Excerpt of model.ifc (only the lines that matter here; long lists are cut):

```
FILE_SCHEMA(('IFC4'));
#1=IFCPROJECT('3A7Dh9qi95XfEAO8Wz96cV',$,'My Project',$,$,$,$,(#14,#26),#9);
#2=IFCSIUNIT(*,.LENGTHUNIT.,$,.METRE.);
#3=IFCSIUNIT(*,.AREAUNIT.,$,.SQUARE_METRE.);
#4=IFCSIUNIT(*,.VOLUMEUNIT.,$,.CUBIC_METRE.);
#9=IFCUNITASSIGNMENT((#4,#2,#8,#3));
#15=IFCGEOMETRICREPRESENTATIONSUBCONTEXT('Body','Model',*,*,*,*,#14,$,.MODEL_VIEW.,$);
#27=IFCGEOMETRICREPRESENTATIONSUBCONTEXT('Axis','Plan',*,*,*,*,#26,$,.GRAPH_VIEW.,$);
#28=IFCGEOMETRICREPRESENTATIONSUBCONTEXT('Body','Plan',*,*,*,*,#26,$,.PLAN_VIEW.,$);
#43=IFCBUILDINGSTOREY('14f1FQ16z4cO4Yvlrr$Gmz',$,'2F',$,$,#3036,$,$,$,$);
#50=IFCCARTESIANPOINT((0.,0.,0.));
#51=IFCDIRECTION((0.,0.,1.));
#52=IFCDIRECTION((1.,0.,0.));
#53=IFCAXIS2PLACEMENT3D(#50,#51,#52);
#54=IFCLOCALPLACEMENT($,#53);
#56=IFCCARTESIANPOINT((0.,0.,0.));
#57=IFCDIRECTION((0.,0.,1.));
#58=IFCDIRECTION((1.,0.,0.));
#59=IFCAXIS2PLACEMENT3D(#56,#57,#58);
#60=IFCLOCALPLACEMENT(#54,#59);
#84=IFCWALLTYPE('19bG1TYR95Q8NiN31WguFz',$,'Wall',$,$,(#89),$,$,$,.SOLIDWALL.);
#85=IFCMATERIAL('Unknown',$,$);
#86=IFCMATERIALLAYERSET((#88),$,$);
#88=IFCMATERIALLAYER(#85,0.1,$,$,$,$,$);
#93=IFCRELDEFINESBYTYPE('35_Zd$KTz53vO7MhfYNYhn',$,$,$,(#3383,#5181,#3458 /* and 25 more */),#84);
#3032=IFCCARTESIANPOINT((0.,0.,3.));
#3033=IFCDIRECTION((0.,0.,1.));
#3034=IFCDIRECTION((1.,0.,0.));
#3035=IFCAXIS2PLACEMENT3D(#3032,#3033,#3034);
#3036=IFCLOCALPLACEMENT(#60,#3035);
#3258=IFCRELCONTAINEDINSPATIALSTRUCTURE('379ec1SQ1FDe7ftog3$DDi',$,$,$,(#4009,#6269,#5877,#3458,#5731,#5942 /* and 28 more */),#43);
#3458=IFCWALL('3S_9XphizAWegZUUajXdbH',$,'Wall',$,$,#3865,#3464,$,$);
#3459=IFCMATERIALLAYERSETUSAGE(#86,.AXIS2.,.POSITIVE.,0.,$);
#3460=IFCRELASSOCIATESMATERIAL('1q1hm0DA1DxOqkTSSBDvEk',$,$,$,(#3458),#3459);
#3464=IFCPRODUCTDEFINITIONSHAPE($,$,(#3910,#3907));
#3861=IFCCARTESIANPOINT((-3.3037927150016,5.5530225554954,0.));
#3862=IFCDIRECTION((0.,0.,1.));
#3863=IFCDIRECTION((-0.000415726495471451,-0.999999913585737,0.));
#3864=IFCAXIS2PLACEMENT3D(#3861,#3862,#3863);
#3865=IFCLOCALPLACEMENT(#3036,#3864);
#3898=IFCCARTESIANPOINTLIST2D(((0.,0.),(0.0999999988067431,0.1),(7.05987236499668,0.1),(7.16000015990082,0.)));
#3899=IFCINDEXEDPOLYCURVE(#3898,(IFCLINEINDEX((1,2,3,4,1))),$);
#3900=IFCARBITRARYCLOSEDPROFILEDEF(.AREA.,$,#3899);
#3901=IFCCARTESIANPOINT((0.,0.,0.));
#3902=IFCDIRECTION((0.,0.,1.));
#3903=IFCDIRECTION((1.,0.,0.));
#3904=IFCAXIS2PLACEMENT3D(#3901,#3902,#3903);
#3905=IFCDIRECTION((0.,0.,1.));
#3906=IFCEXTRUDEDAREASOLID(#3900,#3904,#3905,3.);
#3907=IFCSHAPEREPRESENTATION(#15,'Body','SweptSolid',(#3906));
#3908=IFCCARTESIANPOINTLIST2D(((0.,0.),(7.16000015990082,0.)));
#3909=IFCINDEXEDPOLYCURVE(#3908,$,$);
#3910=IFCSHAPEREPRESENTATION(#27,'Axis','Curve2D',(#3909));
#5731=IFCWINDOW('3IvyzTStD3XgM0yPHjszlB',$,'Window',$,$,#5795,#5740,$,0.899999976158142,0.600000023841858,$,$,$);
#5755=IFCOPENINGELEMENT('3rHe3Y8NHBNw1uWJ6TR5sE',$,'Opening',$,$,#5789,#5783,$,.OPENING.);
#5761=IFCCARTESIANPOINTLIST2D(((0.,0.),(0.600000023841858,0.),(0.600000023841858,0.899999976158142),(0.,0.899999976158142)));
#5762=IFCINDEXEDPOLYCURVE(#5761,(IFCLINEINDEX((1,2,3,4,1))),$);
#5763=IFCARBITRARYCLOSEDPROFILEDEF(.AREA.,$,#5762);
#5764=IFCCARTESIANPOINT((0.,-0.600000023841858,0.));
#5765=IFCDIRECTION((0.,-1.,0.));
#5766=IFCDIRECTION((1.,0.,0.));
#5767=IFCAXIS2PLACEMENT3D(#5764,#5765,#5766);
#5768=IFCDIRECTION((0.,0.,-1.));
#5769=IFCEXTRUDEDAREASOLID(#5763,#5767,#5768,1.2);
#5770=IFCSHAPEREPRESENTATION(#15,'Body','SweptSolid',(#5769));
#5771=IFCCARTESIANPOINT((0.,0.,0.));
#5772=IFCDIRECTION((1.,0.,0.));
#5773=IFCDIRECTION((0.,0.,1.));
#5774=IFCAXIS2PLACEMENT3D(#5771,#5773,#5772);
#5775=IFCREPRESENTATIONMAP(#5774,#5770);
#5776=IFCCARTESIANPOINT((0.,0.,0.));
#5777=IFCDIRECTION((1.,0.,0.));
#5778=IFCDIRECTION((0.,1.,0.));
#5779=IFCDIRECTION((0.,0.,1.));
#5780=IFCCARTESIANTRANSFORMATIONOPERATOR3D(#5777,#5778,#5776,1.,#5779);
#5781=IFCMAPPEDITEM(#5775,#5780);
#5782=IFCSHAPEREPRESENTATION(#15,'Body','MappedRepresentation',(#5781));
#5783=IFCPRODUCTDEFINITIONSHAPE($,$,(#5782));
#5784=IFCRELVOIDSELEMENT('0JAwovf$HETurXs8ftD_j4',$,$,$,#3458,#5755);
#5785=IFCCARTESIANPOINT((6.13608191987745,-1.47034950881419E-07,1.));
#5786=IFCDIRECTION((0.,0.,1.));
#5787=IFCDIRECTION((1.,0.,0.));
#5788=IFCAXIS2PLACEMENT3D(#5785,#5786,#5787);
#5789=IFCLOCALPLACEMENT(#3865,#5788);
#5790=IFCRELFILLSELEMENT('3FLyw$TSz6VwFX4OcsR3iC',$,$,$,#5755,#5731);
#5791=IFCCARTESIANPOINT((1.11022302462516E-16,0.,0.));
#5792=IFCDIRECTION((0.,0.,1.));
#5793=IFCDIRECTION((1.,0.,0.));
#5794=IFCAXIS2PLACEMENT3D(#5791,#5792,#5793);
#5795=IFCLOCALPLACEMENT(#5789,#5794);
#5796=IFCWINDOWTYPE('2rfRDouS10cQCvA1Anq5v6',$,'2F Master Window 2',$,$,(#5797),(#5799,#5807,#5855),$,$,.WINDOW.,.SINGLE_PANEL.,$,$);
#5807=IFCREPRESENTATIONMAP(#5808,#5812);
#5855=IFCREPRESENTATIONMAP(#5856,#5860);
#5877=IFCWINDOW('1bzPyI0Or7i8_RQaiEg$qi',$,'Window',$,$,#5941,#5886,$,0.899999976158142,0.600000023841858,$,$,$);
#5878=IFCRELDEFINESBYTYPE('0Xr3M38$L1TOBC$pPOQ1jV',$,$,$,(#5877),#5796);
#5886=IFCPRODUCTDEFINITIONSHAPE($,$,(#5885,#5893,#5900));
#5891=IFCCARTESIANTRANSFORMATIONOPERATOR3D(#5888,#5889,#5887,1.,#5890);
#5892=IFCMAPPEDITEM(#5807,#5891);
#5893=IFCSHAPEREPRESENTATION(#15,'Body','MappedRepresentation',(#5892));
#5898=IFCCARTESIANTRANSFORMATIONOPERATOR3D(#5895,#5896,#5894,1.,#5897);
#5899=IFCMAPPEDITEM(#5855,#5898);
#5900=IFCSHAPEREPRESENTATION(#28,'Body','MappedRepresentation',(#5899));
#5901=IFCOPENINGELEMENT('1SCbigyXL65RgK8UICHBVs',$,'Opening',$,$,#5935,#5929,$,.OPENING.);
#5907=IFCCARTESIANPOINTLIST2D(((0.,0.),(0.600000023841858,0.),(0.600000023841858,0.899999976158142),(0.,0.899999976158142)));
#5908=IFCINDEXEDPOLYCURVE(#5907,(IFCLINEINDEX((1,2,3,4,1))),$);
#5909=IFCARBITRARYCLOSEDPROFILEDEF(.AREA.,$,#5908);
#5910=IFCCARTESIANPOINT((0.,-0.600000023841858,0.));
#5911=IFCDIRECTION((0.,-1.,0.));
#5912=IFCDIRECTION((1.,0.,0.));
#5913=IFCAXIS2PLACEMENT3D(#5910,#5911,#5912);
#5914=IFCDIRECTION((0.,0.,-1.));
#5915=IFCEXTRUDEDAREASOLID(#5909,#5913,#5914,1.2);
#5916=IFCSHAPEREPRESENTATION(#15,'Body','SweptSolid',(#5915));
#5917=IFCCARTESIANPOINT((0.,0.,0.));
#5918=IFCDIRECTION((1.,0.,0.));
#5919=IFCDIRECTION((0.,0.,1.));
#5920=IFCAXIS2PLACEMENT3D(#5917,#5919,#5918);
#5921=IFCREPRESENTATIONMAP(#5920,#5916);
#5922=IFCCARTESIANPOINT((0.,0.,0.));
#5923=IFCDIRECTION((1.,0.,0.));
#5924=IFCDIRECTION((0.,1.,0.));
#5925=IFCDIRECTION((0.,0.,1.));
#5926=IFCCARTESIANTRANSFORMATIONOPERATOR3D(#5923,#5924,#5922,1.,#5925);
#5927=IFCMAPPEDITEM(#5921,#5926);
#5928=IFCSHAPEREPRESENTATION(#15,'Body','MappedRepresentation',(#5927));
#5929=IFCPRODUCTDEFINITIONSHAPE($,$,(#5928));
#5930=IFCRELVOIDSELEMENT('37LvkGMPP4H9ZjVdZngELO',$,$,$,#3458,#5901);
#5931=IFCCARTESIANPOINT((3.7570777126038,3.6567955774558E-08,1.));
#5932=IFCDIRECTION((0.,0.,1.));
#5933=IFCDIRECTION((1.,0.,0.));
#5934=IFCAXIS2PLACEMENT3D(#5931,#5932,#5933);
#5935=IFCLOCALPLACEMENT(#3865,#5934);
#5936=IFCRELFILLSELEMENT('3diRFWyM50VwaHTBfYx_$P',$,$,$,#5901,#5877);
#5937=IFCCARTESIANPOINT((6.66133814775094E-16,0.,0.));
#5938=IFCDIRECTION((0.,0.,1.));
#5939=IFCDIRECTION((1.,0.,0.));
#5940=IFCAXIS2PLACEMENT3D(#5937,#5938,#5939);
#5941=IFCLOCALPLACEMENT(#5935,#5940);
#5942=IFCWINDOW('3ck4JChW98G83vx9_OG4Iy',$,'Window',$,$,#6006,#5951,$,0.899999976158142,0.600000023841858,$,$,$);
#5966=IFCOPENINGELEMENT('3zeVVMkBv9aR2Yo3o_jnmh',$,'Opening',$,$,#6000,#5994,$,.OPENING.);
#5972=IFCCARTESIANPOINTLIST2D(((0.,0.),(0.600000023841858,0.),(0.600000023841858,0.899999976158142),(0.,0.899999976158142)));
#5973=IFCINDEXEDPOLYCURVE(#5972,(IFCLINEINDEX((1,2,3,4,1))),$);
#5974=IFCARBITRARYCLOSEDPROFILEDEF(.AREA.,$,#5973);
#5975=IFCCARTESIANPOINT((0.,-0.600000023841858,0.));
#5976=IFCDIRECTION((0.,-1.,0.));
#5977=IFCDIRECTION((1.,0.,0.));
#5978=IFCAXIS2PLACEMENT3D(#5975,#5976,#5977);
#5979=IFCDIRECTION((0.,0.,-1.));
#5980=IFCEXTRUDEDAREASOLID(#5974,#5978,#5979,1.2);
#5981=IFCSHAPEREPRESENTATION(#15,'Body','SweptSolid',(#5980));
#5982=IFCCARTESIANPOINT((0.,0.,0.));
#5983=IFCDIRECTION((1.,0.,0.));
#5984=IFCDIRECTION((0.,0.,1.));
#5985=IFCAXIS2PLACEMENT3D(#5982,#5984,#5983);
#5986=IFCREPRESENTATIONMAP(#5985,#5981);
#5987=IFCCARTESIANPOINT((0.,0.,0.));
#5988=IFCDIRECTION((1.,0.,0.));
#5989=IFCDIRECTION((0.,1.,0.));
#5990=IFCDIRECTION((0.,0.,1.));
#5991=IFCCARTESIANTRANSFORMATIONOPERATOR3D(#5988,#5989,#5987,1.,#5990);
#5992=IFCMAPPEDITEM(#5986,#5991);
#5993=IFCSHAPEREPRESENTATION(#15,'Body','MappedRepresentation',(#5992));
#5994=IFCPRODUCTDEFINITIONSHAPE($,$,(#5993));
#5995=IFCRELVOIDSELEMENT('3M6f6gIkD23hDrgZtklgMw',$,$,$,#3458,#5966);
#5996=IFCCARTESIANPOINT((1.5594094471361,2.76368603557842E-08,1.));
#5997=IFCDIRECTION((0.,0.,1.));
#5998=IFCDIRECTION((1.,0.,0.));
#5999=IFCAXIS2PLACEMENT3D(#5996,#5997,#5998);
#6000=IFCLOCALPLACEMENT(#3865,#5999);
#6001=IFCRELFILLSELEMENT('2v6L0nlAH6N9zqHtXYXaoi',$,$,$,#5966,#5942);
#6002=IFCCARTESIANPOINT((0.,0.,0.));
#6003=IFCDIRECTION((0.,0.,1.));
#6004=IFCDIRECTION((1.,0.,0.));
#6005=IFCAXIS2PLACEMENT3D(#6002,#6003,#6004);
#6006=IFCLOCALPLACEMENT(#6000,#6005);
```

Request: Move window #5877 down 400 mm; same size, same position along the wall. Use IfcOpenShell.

```python
import numpy as np
import ifcopenshell
import ifcopenshell.api.geometry
import ifcopenshell.util.placement
import ifcopenshell.util.unit

model = ifcopenshell.open("model.ifc")
unit_scale = ifcopenshell.util.unit.calculate_unit_scale(model)

window = model.by_guid("1bzPyI0Or7i8_RQaiEg$qi")
opening = window.FillsVoids[0].RelatingOpeningElement
dz = -0.4 / unit_scale

shift = np.array([0.0, 0.0, dz])
# The window is placed relative to its opening, so it follows when the opening moves.
matrix = ifcopenshell.util.placement.get_local_placement(opening.ObjectPlacement)
matrix[:3, 3] += shift
ifcopenshell.api.geometry.edit_object_placement(
    model, product=opening, matrix=matrix, is_si=False, should_transform_children=True
)

print(f"moved by {dz * unit_scale:+.3f} m")

model.write("model_v2.ifc")
```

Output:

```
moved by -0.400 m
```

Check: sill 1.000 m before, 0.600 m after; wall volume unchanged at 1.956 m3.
